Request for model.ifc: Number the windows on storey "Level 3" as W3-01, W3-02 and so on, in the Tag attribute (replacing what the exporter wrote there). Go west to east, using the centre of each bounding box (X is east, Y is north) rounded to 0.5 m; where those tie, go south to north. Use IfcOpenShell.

First a look at what the model holds.

```python
import ifcopenshell
import ifcopenshell.util.element
import ifcopenshell.util.placement

model = ifcopenshell.open("model.ifc")
print(model.schema)
storey = next(s for s in model.by_type("IfcBuildingStorey") if s.Name == "Level 3")
windows = [e for e in ifcopenshell.util.element.get_decomposition(storey) if e.is_a("IfcWindow")]
for e in sorted(windows, key=lambda e: e.id()):
    origin = ifcopenshell.util.placement.get_local_placement(e.ObjectPlacement)[:3, 3]
    print(e.id(), e.Tag, e.Name, origin.round(2) + 0.0, sep=" | ")
```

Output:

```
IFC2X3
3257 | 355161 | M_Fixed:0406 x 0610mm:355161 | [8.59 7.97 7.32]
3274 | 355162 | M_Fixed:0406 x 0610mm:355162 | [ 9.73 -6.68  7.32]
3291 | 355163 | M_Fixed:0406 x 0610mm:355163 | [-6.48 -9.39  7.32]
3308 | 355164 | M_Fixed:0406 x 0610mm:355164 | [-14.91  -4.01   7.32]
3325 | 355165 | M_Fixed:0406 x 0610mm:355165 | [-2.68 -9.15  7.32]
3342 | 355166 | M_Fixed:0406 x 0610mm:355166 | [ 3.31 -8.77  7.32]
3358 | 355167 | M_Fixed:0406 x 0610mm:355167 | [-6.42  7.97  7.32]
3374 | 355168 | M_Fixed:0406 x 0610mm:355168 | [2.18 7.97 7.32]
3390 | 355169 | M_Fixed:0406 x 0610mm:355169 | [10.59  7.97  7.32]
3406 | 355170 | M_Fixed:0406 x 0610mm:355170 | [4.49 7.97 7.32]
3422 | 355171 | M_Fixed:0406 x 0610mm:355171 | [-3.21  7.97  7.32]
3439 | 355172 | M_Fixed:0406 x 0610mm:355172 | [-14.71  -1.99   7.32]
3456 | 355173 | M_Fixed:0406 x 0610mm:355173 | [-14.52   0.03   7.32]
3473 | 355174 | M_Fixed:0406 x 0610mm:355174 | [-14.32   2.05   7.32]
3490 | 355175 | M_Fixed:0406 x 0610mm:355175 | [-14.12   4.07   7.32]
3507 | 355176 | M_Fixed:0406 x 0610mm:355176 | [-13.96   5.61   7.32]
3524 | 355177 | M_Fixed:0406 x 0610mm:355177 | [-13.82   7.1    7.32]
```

```python
import ifcopenshell
import ifcopenshell.geom
import ifcopenshell.util.element
import ifcopenshell.util.shape

model = ifcopenshell.open("model.ifc")
settings = ifcopenshell.geom.settings()
settings.set("use-world-coords", True)


def centre(element):
    shape = ifcopenshell.geom.create_shape(settings, element)
    return ifcopenshell.util.shape.get_bbox_centroid(shape.geometry)


storey = next(s for s in model.by_type("IfcBuildingStorey") if s.Name == "Level 3")
windows = [e for e in ifcopenshell.util.element.get_decomposition(storey) if e.is_a("IfcWindow")]

# Insertion points can sit at a corner or the storey origin, so sort by the geometry (in metres).
centres = {e: centre(e) for e in windows}
windows.sort(key=lambda e: (round(centres[e][0] / 0.5), centres[e][1]))

for i, e in enumerate(windows, start=1):
    number = f"W3-{i:02d}"
    e.Tag = number
    print(e.id(), number)

model.write("model_v2.ifc")
```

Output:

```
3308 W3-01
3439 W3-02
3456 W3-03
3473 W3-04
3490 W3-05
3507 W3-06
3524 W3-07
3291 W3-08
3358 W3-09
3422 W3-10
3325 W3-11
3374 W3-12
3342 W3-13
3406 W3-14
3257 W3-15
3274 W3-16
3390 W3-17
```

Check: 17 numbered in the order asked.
